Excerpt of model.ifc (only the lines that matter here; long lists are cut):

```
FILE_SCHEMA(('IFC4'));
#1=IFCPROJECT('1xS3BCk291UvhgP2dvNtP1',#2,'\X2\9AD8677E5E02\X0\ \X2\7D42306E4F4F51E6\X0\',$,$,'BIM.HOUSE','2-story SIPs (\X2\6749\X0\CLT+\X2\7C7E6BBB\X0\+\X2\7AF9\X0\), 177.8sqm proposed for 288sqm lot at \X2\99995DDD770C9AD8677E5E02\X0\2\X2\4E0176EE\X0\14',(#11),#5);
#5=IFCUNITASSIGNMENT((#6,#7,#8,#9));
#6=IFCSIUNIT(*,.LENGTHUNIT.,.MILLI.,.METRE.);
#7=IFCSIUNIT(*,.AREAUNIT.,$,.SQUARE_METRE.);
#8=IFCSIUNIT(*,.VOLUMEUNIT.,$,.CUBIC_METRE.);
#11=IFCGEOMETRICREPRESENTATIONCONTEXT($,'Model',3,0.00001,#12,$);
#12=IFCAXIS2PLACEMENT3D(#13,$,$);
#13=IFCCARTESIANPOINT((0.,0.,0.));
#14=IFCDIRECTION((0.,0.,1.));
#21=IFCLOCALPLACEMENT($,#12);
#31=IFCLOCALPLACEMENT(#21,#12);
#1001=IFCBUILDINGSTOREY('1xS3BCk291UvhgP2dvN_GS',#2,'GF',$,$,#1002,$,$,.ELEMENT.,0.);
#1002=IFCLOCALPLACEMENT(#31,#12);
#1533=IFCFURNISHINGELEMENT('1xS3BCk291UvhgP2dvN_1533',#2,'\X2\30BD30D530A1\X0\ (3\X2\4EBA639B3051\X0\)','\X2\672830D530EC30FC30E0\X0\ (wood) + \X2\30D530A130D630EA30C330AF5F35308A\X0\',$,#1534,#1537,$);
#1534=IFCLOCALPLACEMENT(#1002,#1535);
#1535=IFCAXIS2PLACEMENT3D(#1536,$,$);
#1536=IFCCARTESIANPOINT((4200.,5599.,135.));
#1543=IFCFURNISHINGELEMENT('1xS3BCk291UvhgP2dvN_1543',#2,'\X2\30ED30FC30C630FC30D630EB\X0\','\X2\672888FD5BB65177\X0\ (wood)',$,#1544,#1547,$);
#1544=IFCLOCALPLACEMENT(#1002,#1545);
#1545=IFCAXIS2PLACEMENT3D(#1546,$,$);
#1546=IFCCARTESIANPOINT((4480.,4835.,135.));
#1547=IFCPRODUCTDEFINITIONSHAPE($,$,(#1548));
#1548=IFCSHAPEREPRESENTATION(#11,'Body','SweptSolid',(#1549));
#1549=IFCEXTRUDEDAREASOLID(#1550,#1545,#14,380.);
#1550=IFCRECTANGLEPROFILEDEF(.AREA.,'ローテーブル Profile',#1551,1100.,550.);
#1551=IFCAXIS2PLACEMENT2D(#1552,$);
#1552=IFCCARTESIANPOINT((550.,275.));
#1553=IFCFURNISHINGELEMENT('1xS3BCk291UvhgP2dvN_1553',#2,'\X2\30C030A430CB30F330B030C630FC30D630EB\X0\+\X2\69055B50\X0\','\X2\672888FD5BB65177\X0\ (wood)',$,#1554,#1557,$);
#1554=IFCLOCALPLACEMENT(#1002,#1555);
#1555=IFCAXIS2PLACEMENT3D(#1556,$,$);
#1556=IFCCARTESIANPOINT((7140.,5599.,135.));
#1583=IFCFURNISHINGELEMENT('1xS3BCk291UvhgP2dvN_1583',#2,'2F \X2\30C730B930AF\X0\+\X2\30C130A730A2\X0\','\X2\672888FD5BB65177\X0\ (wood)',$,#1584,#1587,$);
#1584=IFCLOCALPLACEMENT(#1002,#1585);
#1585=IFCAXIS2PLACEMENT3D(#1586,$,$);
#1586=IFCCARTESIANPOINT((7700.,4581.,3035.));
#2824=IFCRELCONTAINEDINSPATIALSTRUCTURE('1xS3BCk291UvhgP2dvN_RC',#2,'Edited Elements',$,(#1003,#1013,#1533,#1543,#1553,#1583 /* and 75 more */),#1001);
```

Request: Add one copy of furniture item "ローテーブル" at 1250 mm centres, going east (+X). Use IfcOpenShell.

```python
import numpy as np
import ifcopenshell
import ifcopenshell.api.geometry
import ifcopenshell.api.root
import ifcopenshell.util.element
import ifcopenshell.util.placement
import ifcopenshell.util.unit

model = ifcopenshell.open("model.ifc")
unit_scale = ifcopenshell.util.unit.calculate_unit_scale(model)


def reuse_history(source, copy):
    """copy_class also copies each property set's owner history, people and application; keep the originals."""
    for rel in copy.IsDefinedBy:
        if rel.is_a("IfcRelDefinesByProperties") and (history := rel.RelatingPropertyDefinition.OwnerHistory):
            rel.RelatingPropertyDefinition.OwnerHistory = source.OwnerHistory
            ifcopenshell.util.element.remove_deep2(model, history)


source = model.by_guid("1xS3BCk291UvhgP2dvN_1543")
base = ifcopenshell.util.placement.get_local_placement(source.ObjectPlacement)
step = np.array([1.0, 0.0, 0.0]) * 1.25 / unit_scale

for i in range(1, 2):
    copy = ifcopenshell.api.root.copy_class(model, product=source)
    copy.Representation = ifcopenshell.util.element.copy_deep(
        model, source.Representation, exclude=["IfcGeometricRepresentationContext", "IfcRepresentationMap"]
    )
    reuse_history(source, copy)
    matrix = base.copy()
    matrix[:3, 3] += i * step
    print("added at", matrix[:3, 3].round(3) + 0.0)
    ifcopenshell.api.geometry.edit_object_placement(model, product=copy, matrix=matrix, is_si=False)

model.write("model_edited.ifc")
```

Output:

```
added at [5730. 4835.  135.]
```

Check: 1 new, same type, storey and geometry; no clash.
